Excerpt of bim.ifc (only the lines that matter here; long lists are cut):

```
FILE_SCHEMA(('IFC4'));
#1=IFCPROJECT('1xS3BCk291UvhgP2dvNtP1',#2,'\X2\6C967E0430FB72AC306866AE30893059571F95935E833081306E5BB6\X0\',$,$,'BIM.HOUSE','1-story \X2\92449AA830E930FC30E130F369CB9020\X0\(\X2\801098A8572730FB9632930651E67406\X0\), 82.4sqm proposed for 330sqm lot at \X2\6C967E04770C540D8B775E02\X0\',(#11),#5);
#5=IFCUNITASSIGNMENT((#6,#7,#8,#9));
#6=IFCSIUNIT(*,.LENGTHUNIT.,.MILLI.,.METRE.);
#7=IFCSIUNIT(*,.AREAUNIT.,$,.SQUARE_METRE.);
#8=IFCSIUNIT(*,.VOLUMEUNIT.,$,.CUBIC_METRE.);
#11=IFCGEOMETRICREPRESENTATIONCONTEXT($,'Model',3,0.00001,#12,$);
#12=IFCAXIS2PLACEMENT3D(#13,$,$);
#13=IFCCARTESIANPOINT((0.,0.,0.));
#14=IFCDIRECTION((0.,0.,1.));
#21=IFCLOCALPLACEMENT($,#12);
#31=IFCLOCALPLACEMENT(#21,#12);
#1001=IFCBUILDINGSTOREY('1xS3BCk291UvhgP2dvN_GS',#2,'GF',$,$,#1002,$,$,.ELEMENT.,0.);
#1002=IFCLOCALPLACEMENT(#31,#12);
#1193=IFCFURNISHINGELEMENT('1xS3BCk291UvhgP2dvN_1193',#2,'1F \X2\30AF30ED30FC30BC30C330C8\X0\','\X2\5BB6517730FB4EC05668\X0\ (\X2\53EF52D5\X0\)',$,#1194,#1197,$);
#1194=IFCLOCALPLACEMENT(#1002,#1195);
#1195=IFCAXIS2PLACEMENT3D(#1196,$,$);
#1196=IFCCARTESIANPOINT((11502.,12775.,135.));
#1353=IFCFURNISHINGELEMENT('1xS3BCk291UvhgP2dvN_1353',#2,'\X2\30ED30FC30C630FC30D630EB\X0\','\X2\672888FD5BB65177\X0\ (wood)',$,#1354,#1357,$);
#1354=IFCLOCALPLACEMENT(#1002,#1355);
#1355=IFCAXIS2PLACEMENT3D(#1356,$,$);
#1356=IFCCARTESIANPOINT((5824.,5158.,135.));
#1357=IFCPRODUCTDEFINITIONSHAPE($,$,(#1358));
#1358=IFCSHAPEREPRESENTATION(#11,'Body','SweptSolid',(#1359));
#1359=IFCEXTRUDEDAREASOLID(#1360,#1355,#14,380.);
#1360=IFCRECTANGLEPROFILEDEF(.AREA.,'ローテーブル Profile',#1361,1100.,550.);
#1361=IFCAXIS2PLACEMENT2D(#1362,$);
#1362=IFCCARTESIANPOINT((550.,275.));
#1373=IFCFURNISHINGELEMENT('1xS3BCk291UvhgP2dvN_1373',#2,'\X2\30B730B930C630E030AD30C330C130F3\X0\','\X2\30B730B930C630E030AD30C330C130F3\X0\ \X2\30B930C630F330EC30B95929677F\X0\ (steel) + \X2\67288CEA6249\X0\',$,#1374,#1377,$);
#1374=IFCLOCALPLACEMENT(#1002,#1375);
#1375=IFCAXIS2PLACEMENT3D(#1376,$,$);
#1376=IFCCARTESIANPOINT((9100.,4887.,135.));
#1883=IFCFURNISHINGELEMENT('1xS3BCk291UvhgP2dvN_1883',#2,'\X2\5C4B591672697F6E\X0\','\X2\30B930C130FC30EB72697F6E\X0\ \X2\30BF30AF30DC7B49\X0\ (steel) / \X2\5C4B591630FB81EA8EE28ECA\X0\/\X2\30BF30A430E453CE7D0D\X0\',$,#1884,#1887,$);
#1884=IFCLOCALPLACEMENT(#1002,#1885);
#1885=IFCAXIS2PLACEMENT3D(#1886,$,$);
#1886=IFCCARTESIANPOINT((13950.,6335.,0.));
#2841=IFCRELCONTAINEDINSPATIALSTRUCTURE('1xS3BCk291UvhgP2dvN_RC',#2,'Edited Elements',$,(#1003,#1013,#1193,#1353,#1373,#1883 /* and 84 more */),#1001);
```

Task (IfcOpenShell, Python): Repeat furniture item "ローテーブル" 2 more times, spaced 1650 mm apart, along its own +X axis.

```python
import ifcopenshell
import ifcopenshell.api.geometry
import ifcopenshell.api.root
import ifcopenshell.util.element
import ifcopenshell.util.placement
import ifcopenshell.util.unit

model = ifcopenshell.open("bim.ifc")
unit_scale = ifcopenshell.util.unit.calculate_unit_scale(model)


def reuse_history(source, copy):
    """copy_class also copies each property set's owner history, people and application; keep the originals."""
    for rel in copy.IsDefinedBy:
        if rel.is_a("IfcRelDefinesByProperties") and (history := rel.RelatingPropertyDefinition.OwnerHistory):
            rel.RelatingPropertyDefinition.OwnerHistory = source.OwnerHistory
            ifcopenshell.util.element.remove_deep2(model, history)


source = model.by_id(1353)
base = ifcopenshell.util.placement.get_local_placement(source.ObjectPlacement)
step = base[:3, 0] * 1.65 / unit_scale

for i in range(1, 3):
    copy = ifcopenshell.api.root.copy_class(model, product=source)
    copy.Representation = ifcopenshell.util.element.copy_deep(
        model, source.Representation, exclude=["IfcGeometricRepresentationContext", "IfcRepresentationMap"]
    )
    reuse_history(source, copy)
    matrix = base.copy()
    matrix[:3, 3] += i * step
    print("added at", matrix[:3, 3].round(3) + 0.0)
    ifcopenshell.api.geometry.edit_object_placement(model, product=copy, matrix=matrix, is_si=False)

model.write("bim-out.ifc")
```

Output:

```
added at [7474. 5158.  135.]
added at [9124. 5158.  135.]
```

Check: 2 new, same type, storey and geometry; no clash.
